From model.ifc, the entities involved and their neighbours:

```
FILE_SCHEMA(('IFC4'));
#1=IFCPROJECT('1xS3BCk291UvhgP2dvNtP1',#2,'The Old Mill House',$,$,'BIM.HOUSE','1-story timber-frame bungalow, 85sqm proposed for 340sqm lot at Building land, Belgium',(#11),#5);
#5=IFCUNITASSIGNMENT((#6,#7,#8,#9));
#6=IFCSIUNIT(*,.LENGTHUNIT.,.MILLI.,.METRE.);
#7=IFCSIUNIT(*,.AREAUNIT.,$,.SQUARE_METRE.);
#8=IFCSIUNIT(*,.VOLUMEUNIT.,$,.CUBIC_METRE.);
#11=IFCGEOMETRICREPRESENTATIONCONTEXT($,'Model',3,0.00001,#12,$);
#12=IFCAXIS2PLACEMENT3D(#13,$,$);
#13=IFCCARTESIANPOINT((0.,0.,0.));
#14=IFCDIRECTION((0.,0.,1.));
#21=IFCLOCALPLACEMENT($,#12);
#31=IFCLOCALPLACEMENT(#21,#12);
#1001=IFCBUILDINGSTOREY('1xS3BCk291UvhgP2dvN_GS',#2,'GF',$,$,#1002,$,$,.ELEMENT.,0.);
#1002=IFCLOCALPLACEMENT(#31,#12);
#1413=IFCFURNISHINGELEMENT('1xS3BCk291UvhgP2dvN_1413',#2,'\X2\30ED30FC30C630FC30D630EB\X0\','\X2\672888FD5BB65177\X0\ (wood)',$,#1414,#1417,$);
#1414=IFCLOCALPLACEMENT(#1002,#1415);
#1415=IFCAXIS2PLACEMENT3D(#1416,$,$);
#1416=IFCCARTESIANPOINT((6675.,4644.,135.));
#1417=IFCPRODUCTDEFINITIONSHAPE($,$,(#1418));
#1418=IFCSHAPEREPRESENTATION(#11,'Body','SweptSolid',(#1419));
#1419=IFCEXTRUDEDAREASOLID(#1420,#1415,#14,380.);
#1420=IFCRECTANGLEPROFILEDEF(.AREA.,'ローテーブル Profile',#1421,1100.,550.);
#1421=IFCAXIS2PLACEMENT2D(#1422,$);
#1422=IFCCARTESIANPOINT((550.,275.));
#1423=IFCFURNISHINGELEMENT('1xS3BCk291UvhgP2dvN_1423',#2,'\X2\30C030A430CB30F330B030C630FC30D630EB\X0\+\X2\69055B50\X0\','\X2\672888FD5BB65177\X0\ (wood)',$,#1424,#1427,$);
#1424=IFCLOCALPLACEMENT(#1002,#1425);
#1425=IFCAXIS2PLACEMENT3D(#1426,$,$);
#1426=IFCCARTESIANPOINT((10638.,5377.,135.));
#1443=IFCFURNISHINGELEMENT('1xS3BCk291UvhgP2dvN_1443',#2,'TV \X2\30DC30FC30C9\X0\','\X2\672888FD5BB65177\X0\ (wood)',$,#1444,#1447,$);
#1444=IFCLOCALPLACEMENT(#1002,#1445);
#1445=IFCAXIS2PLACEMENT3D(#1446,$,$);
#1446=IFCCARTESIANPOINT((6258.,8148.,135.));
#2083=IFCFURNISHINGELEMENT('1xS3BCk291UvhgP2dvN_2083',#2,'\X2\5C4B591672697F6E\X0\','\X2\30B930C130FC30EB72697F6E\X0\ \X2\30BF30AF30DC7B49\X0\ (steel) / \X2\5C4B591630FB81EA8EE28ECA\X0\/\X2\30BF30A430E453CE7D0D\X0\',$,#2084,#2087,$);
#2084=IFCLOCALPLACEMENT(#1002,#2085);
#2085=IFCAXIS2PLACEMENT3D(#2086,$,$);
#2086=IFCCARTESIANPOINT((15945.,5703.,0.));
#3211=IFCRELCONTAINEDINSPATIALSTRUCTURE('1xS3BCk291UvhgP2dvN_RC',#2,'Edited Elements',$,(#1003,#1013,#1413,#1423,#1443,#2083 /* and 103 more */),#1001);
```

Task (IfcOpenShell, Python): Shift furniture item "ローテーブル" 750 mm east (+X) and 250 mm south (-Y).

```python
import ifcopenshell
import ifcopenshell.api.geometry
import ifcopenshell.util.placement

model = ifcopenshell.open("model.ifc")

item = model.by_id(1413)
matrix = ifcopenshell.util.placement.get_local_placement(item.ObjectPlacement)
matrix[0, 3] += 750.0
matrix[1, 3] -= 250.0
ifcopenshell.api.geometry.edit_object_placement(model, product=item, matrix=matrix, is_si=False)

print(ifcopenshell.util.placement.get_local_placement(item.ObjectPlacement).round(3) + 0.0)

model.write("model_updated.ifc")
```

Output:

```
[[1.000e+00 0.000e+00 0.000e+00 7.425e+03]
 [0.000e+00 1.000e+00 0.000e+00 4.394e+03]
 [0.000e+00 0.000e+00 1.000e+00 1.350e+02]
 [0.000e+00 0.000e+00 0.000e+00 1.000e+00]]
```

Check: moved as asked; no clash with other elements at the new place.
